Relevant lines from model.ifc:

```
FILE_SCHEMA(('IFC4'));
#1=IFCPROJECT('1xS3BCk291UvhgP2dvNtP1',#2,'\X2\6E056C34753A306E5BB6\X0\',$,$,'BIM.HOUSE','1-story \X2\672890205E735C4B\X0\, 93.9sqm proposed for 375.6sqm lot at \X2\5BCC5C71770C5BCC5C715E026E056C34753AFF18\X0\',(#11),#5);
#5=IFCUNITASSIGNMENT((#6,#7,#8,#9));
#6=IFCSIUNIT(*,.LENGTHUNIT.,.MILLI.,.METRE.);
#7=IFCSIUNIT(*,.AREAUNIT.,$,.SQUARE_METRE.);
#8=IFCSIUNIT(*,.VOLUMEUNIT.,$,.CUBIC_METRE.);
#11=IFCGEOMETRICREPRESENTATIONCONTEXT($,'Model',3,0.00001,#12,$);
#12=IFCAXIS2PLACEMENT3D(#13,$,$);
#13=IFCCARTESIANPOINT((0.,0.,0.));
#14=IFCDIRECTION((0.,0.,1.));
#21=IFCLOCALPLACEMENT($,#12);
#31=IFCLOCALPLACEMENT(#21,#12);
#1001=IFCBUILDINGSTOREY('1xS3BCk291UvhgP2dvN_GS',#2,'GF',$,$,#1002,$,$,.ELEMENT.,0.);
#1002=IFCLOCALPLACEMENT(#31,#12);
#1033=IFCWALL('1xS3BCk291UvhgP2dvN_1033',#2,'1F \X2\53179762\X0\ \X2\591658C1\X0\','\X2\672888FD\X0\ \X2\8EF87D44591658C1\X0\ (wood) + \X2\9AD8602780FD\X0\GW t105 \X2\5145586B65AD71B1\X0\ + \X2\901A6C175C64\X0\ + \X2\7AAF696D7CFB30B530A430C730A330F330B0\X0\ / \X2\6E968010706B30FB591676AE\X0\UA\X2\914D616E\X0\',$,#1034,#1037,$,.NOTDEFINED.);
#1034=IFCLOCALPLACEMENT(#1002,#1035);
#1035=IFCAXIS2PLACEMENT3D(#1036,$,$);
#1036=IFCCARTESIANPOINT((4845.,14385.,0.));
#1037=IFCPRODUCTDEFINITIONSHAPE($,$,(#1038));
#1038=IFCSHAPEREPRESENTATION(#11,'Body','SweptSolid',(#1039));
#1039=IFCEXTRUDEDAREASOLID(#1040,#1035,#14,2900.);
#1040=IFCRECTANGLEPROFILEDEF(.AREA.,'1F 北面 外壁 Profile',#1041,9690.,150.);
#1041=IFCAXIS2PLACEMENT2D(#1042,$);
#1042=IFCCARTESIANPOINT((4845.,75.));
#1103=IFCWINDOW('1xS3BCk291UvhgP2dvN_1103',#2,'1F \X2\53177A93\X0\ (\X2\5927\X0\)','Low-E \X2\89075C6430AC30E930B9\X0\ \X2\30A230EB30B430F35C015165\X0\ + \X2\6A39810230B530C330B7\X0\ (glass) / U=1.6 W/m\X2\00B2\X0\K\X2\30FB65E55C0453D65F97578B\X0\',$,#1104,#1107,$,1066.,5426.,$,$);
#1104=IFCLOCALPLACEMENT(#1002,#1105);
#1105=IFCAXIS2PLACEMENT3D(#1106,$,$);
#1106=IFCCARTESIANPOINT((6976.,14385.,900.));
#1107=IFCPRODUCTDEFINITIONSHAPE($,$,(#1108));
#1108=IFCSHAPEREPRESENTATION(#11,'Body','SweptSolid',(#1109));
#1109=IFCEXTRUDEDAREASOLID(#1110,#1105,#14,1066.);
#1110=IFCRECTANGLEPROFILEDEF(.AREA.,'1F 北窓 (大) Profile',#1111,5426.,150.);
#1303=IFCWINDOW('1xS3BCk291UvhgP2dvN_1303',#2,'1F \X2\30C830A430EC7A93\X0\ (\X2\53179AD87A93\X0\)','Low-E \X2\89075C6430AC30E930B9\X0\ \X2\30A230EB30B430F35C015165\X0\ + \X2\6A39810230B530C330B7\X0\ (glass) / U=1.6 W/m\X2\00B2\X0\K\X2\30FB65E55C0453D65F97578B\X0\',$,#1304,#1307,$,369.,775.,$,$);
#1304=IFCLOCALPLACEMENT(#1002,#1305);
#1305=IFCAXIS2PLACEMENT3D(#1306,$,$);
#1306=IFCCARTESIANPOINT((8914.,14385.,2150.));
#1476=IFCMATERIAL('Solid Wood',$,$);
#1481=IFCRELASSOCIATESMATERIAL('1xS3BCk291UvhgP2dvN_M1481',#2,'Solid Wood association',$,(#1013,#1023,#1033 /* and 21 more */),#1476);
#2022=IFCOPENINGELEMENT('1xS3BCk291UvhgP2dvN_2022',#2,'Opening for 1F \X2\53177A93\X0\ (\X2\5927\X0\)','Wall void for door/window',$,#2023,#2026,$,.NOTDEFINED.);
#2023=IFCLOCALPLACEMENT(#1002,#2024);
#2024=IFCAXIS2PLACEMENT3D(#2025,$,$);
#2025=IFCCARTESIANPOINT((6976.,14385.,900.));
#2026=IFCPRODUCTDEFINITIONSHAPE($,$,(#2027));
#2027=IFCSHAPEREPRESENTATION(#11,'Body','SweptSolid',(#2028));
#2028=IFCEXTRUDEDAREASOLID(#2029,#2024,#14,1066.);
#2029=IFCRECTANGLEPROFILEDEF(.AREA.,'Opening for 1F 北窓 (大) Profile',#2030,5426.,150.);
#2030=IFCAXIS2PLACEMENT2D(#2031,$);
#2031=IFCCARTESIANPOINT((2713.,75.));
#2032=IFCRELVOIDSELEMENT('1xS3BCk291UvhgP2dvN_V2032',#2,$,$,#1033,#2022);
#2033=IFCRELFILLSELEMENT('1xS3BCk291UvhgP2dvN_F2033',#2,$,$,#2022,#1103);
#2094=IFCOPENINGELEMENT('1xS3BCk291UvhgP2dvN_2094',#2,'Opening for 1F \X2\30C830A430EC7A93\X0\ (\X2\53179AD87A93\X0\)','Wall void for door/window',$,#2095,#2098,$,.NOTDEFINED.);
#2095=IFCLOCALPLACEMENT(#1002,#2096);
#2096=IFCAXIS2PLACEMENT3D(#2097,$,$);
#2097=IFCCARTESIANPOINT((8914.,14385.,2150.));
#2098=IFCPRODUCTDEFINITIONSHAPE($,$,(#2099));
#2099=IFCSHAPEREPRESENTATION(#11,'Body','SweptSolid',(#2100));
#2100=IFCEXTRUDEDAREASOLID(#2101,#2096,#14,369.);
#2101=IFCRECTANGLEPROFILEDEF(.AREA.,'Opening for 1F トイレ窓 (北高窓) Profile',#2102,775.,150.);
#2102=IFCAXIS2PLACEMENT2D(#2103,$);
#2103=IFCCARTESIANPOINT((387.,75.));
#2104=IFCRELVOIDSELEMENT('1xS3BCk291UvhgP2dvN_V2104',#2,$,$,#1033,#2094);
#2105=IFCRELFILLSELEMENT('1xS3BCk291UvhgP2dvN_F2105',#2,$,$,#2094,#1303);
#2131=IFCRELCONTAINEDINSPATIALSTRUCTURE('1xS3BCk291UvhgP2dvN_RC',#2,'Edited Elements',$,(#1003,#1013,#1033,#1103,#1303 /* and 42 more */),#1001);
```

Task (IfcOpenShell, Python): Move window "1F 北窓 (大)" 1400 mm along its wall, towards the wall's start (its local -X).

```python
import ifcopenshell
import ifcopenshell.api.geometry
import ifcopenshell.util.placement

model = ifcopenshell.open("model.ifc")

window = model.by_id(1103)
opening = window.FillsVoids[0].RelatingOpeningElement
wall = opening.VoidsElements[0].RelatingBuildingElement

wall_matrix = ifcopenshell.util.placement.get_local_placement(wall.ObjectPlacement)
shift = wall_matrix[:3, 0] * -1400.0
before = ifcopenshell.util.placement.get_local_placement(window.ObjectPlacement)[:3, 3].copy()

# The window is not placed relative to its opening, so move both.
for product in (opening, window):
    matrix = ifcopenshell.util.placement.get_local_placement(product.ObjectPlacement)
    matrix[:3, 3] += shift
    ifcopenshell.api.geometry.edit_object_placement(model, product=product, matrix=matrix, is_si=False)

after = ifcopenshell.util.placement.get_local_placement(window.ObjectPlacement)[:3, 3]
print("window moved by", (after - before).round(3) + 0.0)

model.write("model_edited.ifc")
```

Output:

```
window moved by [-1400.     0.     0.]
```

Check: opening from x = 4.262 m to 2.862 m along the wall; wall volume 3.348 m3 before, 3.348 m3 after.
